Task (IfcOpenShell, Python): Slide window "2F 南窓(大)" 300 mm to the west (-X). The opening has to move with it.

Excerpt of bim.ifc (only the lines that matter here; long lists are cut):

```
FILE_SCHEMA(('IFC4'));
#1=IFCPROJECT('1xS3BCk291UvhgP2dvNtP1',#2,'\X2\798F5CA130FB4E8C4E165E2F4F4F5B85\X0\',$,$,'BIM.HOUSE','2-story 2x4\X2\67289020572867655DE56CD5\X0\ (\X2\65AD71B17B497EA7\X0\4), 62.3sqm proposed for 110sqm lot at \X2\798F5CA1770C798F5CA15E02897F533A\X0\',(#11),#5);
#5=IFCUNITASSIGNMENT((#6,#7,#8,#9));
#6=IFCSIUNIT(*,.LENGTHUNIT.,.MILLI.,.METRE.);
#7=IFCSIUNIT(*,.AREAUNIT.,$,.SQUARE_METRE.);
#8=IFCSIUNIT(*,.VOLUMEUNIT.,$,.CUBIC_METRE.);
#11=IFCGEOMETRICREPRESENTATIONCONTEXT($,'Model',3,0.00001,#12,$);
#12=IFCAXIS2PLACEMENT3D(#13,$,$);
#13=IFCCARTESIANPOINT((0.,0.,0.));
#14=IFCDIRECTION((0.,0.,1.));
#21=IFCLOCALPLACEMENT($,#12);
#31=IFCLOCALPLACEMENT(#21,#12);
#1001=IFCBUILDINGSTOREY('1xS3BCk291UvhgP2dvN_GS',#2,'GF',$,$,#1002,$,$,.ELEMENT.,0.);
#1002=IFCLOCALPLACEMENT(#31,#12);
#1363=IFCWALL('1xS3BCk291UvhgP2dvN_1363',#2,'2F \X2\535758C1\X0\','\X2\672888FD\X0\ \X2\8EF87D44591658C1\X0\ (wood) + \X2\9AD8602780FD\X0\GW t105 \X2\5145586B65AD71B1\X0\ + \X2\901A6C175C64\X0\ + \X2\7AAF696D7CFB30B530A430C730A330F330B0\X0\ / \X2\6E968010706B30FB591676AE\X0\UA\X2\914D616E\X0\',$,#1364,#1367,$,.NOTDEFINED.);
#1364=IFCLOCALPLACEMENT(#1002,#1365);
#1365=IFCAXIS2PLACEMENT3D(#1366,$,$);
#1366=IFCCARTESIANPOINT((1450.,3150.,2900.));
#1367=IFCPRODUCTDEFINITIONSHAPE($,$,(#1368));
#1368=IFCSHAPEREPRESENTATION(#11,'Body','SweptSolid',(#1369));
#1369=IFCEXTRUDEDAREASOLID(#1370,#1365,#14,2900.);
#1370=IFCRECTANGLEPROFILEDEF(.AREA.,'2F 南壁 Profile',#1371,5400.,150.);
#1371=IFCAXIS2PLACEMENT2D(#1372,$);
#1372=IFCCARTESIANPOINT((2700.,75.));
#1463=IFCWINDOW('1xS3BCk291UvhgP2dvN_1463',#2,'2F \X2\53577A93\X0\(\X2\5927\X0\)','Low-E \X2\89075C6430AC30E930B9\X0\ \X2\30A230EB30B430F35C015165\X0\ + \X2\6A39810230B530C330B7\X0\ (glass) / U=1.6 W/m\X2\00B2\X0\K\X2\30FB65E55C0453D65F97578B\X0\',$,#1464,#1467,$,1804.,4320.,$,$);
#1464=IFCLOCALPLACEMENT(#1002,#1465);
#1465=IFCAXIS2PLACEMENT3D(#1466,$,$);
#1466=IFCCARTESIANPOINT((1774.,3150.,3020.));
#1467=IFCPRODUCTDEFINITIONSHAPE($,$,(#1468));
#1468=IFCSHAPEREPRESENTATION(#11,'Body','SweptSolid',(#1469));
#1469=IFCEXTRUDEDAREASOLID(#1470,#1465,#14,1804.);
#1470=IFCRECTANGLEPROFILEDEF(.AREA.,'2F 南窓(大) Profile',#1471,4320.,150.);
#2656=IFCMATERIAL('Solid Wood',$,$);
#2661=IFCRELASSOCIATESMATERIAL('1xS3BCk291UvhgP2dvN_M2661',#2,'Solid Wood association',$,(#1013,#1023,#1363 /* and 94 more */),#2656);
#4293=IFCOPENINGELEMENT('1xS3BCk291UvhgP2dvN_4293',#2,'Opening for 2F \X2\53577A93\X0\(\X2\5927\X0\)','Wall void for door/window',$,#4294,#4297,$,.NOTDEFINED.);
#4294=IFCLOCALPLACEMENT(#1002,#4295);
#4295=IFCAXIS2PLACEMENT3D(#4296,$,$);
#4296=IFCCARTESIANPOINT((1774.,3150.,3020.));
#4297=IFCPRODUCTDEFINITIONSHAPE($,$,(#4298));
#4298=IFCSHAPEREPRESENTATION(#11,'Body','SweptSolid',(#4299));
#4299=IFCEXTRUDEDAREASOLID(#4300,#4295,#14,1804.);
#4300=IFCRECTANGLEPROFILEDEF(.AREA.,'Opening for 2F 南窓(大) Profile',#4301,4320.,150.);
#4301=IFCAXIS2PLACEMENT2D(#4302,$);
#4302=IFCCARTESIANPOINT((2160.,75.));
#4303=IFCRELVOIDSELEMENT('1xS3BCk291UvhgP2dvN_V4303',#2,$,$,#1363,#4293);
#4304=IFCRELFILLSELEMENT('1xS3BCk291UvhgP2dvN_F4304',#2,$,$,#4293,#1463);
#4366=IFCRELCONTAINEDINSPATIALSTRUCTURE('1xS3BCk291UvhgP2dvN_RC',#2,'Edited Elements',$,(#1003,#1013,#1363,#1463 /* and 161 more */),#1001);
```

```python
import ifcopenshell
import ifcopenshell.api.geometry
import ifcopenshell.util.placement
import ifcopenshell.util.unit

model = ifcopenshell.open("bim.ifc")
unit_scale = ifcopenshell.util.unit.calculate_unit_scale(model)

window = model.by_guid("1xS3BCk291UvhgP2dvN_1463")
opening = window.FillsVoids[0].RelatingOpeningElement
wall = opening.VoidsElements[0].RelatingBuildingElement

wall_matrix = ifcopenshell.util.placement.get_local_placement(wall.ObjectPlacement)
shift = wall_matrix[:3, 0] * -0.3 / unit_scale
before = ifcopenshell.util.placement.get_local_placement(window.ObjectPlacement)[:3, 3].copy()

# The window is not placed relative to its opening, so move both.
for product in (opening, window):
    matrix = ifcopenshell.util.placement.get_local_placement(product.ObjectPlacement)
    matrix[:3, 3] += shift
    ifcopenshell.api.geometry.edit_object_placement(model, product=product, matrix=matrix, is_si=False)

after = ifcopenshell.util.placement.get_local_placement(window.ObjectPlacement)[:3, 3]
print("window moved by", (after - before).round(3) + 0.0)

model.write("bim-out.ifc")
```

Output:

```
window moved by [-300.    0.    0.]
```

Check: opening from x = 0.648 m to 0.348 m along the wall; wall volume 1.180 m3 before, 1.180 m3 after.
